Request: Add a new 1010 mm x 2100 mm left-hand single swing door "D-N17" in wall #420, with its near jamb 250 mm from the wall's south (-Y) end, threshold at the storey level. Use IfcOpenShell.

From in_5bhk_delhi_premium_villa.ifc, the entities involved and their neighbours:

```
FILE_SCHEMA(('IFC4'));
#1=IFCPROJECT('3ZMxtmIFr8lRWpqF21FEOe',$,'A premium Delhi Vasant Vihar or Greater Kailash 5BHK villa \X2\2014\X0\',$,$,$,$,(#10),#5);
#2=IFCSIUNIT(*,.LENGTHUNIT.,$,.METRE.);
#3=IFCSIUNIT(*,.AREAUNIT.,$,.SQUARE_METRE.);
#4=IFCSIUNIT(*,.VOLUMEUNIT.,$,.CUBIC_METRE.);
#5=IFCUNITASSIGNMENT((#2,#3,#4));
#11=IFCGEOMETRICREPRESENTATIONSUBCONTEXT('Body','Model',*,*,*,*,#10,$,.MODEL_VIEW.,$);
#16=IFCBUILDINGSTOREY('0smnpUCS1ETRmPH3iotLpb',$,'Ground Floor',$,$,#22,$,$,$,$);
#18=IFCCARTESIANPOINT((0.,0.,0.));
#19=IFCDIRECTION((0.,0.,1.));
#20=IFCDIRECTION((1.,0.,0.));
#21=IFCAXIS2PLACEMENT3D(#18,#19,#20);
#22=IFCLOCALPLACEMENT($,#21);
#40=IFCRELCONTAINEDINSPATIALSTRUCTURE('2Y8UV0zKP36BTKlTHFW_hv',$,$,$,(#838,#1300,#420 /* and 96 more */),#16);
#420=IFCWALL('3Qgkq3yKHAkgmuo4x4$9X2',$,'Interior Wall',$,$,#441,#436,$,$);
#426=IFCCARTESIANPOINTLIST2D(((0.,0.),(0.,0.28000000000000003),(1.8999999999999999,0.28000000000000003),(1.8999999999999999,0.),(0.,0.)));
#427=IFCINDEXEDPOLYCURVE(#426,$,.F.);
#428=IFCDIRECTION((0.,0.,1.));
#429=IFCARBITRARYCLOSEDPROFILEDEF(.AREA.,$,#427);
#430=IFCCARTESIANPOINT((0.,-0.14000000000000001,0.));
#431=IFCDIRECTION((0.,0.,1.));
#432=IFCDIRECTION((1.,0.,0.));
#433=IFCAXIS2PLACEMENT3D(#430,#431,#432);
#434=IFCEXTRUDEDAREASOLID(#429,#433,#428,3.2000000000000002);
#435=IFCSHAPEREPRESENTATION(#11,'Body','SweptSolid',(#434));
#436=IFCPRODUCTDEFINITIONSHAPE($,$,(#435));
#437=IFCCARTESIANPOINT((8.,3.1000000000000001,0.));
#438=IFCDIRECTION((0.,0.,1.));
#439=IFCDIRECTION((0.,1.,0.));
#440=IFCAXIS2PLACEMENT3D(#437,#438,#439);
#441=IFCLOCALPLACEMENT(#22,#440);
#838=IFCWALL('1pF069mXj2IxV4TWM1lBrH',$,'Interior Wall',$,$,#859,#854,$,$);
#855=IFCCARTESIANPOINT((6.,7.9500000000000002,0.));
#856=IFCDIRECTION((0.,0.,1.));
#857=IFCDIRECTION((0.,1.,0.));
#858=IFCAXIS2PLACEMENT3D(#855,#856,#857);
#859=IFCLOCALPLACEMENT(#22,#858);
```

```python
import numpy as np
import ifcopenshell
import ifcopenshell.api.feature
import ifcopenshell.api.geometry
import ifcopenshell.api.root
import ifcopenshell.api.spatial
import ifcopenshell.geom
import ifcopenshell.util.element
import ifcopenshell.util.placement
import ifcopenshell.util.representation
import ifcopenshell.util.shape
import ifcopenshell.util.unit

model = ifcopenshell.open("in_5bhk_delhi_premium_villa.ifc")
unit_scale = ifcopenshell.util.unit.calculate_unit_scale(model)
settings = ifcopenshell.geom.settings()


def volume(element):
    """Net volume in cubic metres, openings subtracted."""
    shape = ifcopenshell.geom.create_shape(settings, element)
    return ifcopenshell.util.shape.get_volume(shape.geometry)


wall = model.by_guid("3Qgkq3yKHAkgmuo4x4$9X2")
storey = ifcopenshell.util.element.get_container(wall, ifc_class="IfcBuildingStorey")
context = ifcopenshell.util.representation.get_context(model, "Model", "Body", "MODEL_VIEW")
before = volume(wall)

width, height, from_end, sill = 1.01, 2.1, 0.25, 0.0  # metres

# The wall runs along its own X axis, and the end named is its -X end.
wall_shape = ifcopenshell.geom.create_shape(settings, wall)
x, y, z = ifcopenshell.util.shape.get_vertices(wall_shape.geometry).T
start = x.min() + from_end
face, thickness = float(y.min()), float(y.max() - y.min())
wall_matrix = ifcopenshell.util.placement.get_local_placement(wall.ObjectPlacement)
level = ifcopenshell.util.placement.get_local_placement(storey.ObjectPlacement)[2, 3]


def in_wall(x, y):
    """Placement at x, y metres in the wall's axes, at sill height."""
    matrix = wall_matrix.copy()
    matrix[:, 3] = wall_matrix @ np.array([x / unit_scale, y / unit_scale, 0.0, 1.0])
    matrix[2, 3] = level + sill / unit_scale
    return matrix


# Opening: a box that overshoots both wall faces by 50 mm.
opening = ifcopenshell.api.root.create_entity(model, ifc_class="IfcOpeningElement", predefined_type="OPENING")
box = ifcopenshell.api.geometry.add_wall_representation(
    model, context=context, length=width, height=height, thickness=thickness + 0.1
)
ifcopenshell.api.geometry.assign_representation(model, product=opening, representation=box)
ifcopenshell.api.geometry.edit_object_placement(model, product=opening, matrix=in_wall(start, face - 0.05), is_si=False)
ifcopenshell.api.feature.add_feature(model, feature=opening, element=wall)

door = ifcopenshell.api.root.create_entity(model, ifc_class="IfcDoor", name="D-N17", predefined_type="DOOR")
door.OverallWidth, door.OverallHeight = width / unit_scale, height / unit_scale
door.OperationType = "SINGLE_SWING_LEFT"
body = ifcopenshell.api.geometry.add_door_representation(
    model,
    context=context,
    overall_width=door.OverallWidth,
    overall_height=door.OverallHeight,
    operation_type="SINGLE_SWING_LEFT",
    lining_properties={"LiningDepth": thickness / unit_scale, "ThresholdDepth": thickness / unit_scale},
)
ifcopenshell.api.geometry.assign_representation(model, product=door, representation=body)
ifcopenshell.api.spatial.assign_container(model, products=[door], relating_structure=storey)
ifcopenshell.api.feature.add_filling(model, opening=opening, element=door)

# The lining spans the wall, so the door starts at the wall face.
ifcopenshell.api.geometry.edit_object_placement(model, product=door, matrix=in_wall(start, face), is_si=False)

after = volume(wall)

print(f"wall volume {before:.3f} -> {after:.3f} m3")

model.write("in_5bhk_delhi_premium_villa_edited.ifc")
```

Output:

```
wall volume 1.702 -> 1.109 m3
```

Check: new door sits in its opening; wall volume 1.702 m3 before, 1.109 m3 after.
